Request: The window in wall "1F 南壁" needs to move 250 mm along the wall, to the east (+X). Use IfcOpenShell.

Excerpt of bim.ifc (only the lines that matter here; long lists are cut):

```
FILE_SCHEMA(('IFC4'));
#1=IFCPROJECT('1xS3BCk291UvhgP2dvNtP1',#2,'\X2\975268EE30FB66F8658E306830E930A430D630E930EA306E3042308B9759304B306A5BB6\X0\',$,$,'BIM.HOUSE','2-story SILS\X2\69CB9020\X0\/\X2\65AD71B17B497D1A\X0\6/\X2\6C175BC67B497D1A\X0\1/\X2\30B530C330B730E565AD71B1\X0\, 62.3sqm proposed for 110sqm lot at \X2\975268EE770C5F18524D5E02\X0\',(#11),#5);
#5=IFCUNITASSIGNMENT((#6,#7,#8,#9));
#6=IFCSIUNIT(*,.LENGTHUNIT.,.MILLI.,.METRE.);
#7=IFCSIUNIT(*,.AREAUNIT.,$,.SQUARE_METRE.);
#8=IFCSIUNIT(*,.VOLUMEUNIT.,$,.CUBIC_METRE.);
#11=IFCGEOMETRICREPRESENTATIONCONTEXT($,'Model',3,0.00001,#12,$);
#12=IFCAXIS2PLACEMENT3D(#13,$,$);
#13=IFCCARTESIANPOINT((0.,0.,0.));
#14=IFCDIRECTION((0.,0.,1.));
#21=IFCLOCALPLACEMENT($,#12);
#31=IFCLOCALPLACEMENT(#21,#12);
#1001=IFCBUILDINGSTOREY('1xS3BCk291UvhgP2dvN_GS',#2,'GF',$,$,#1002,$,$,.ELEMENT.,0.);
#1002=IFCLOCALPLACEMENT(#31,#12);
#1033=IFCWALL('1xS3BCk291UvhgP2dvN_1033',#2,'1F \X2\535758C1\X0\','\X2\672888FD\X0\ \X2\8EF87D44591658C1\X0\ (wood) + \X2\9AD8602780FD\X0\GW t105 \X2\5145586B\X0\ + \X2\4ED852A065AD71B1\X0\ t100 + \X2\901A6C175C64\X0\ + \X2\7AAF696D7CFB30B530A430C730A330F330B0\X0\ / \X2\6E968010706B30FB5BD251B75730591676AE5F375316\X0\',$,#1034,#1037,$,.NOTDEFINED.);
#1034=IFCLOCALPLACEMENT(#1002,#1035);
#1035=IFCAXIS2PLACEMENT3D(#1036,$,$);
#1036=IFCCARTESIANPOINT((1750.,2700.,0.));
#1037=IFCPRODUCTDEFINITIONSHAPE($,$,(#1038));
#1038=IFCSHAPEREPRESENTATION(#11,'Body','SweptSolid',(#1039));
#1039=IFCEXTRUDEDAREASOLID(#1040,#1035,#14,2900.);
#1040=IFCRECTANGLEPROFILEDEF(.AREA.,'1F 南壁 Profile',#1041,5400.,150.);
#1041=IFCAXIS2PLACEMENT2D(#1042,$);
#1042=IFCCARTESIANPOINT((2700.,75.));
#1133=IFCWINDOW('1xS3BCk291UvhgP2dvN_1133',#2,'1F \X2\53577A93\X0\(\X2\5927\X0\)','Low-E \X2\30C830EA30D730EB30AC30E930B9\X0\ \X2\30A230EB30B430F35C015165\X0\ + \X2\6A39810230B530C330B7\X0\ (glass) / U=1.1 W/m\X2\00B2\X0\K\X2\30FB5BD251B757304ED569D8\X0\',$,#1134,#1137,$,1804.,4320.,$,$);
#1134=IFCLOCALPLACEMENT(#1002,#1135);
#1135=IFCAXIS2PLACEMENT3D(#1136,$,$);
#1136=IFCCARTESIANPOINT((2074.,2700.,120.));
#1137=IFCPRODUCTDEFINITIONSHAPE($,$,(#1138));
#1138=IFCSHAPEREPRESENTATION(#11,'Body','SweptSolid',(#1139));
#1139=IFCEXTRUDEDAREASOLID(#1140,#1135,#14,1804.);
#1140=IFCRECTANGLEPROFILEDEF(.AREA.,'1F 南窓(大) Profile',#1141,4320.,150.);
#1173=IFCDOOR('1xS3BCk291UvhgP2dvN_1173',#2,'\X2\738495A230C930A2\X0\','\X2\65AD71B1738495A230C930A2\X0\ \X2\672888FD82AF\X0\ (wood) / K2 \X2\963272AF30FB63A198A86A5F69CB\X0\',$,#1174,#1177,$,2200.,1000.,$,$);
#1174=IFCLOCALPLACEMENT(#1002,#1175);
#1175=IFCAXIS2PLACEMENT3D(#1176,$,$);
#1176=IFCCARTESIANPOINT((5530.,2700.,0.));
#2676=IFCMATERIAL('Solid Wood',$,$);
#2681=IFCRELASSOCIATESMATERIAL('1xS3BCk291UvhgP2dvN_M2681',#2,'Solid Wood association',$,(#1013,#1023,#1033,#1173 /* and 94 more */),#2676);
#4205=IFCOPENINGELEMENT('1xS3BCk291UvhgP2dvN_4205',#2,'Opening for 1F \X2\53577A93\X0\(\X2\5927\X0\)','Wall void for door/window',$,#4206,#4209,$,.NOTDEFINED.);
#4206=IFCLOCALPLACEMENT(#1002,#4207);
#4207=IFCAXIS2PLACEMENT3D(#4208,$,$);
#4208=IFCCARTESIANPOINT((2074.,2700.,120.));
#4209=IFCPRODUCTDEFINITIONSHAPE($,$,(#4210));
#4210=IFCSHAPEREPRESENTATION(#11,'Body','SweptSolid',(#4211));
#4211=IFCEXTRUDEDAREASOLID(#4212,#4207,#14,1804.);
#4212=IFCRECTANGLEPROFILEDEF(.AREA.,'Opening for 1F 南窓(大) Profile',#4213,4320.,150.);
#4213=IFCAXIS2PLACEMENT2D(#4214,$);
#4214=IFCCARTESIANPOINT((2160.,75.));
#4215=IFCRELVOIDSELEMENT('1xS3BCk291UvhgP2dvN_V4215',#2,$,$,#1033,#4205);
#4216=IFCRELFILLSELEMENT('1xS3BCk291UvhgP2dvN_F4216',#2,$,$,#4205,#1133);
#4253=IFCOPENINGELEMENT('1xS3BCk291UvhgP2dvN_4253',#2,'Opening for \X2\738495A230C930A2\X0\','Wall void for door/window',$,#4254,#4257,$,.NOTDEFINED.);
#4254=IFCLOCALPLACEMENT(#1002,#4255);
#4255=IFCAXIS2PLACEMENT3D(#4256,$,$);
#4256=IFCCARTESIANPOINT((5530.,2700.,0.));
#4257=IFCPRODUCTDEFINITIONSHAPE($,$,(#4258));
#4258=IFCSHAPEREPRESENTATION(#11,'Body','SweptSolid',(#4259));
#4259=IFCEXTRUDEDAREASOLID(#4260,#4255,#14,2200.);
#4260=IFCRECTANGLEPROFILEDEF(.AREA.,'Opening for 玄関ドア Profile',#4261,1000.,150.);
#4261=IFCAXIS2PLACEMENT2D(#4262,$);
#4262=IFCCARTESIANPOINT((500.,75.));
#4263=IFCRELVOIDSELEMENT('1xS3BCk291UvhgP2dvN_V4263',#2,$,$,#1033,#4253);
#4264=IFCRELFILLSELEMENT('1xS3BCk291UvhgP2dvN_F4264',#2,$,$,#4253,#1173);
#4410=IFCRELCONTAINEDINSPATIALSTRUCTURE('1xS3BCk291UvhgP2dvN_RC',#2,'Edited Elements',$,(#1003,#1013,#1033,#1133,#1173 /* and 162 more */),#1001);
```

```python
import ifcopenshell
import ifcopenshell.api.geometry
import ifcopenshell.util.placement
import ifcopenshell.util.unit

model = ifcopenshell.open("bim.ifc")
unit_scale = ifcopenshell.util.unit.calculate_unit_scale(model)

window = model.by_guid("1xS3BCk291UvhgP2dvN_1133")
opening = window.FillsVoids[0].RelatingOpeningElement
wall = opening.VoidsElements[0].RelatingBuildingElement

wall_matrix = ifcopenshell.util.placement.get_local_placement(wall.ObjectPlacement)
shift = wall_matrix[:3, 0] * 0.25 / unit_scale
before = ifcopenshell.util.placement.get_local_placement(window.ObjectPlacement)[:3, 3].copy()

# The window is not placed relative to its opening, so move both.
for product in (opening, window):
    matrix = ifcopenshell.util.placement.get_local_placement(product.ObjectPlacement)
    matrix[:3, 3] += shift
    ifcopenshell.api.geometry.edit_object_placement(model, product=product, matrix=matrix, is_si=False)

after = ifcopenshell.util.placement.get_local_placement(window.ObjectPlacement)[:3, 3]
print("window moved by", (after - before).round(3) + 0.0)

model.write("bim_rev.ifc")
```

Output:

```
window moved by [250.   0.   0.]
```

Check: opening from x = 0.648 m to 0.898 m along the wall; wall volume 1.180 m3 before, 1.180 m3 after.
